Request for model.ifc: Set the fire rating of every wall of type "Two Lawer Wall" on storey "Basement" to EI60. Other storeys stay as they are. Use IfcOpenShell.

First a look at what the model holds.

```python
import ifcopenshell
import ifcopenshell.util.element

model = ifcopenshell.open("model.ifc")
print(model.schema)
storey = next(s for s in model.by_type("IfcBuildingStorey") if s.Name == "Basement")
walls = [e for e in ifcopenshell.util.element.get_decomposition(storey) if e.is_a("IfcWall")]
seen = {}
for e in walls:
    element_type = ifcopenshell.util.element.get_type(e)
    key = (element_type.Name if element_type != e and element_type else None, ifcopenshell.util.element.get_pset(e, "Pset_WallCommon", "FireRating"))
    seen[key] = seen.get(key, 0) + 1
for (name, value), count in sorted(seen.items(), key=str):
    print(count, "x", name, "|", value)
```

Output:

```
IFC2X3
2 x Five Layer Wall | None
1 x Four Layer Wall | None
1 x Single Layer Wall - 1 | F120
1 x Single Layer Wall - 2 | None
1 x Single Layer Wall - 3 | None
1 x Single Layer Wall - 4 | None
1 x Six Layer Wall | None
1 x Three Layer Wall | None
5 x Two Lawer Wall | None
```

```python
import ifcopenshell
import ifcopenshell.api.pset
import ifcopenshell.util.element

model = ifcopenshell.open("model.ifc")

storey = next(s for s in model.by_type("IfcBuildingStorey") if s.Name == "Basement")
walls = [e for e in ifcopenshell.util.element.get_decomposition(storey) if e.is_a("IfcWall")]

count = 0
for e in walls:
    element_type = ifcopenshell.util.element.get_type(e)
    if element_type in (None, e) or element_type.Name != "Two Lawer Wall":
        continue
    # add_pset returns the element's existing set when there is one.
    pset = ifcopenshell.api.pset.add_pset(model, product=e, name="Pset_WallCommon")
    ifcopenshell.api.pset.edit_pset(model, pset=pset, properties={"FireRating": "EI60"})
    count += 1

print(count, "walls updated")

model.write("model-out.ifc")
```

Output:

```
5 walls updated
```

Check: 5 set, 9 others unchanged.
